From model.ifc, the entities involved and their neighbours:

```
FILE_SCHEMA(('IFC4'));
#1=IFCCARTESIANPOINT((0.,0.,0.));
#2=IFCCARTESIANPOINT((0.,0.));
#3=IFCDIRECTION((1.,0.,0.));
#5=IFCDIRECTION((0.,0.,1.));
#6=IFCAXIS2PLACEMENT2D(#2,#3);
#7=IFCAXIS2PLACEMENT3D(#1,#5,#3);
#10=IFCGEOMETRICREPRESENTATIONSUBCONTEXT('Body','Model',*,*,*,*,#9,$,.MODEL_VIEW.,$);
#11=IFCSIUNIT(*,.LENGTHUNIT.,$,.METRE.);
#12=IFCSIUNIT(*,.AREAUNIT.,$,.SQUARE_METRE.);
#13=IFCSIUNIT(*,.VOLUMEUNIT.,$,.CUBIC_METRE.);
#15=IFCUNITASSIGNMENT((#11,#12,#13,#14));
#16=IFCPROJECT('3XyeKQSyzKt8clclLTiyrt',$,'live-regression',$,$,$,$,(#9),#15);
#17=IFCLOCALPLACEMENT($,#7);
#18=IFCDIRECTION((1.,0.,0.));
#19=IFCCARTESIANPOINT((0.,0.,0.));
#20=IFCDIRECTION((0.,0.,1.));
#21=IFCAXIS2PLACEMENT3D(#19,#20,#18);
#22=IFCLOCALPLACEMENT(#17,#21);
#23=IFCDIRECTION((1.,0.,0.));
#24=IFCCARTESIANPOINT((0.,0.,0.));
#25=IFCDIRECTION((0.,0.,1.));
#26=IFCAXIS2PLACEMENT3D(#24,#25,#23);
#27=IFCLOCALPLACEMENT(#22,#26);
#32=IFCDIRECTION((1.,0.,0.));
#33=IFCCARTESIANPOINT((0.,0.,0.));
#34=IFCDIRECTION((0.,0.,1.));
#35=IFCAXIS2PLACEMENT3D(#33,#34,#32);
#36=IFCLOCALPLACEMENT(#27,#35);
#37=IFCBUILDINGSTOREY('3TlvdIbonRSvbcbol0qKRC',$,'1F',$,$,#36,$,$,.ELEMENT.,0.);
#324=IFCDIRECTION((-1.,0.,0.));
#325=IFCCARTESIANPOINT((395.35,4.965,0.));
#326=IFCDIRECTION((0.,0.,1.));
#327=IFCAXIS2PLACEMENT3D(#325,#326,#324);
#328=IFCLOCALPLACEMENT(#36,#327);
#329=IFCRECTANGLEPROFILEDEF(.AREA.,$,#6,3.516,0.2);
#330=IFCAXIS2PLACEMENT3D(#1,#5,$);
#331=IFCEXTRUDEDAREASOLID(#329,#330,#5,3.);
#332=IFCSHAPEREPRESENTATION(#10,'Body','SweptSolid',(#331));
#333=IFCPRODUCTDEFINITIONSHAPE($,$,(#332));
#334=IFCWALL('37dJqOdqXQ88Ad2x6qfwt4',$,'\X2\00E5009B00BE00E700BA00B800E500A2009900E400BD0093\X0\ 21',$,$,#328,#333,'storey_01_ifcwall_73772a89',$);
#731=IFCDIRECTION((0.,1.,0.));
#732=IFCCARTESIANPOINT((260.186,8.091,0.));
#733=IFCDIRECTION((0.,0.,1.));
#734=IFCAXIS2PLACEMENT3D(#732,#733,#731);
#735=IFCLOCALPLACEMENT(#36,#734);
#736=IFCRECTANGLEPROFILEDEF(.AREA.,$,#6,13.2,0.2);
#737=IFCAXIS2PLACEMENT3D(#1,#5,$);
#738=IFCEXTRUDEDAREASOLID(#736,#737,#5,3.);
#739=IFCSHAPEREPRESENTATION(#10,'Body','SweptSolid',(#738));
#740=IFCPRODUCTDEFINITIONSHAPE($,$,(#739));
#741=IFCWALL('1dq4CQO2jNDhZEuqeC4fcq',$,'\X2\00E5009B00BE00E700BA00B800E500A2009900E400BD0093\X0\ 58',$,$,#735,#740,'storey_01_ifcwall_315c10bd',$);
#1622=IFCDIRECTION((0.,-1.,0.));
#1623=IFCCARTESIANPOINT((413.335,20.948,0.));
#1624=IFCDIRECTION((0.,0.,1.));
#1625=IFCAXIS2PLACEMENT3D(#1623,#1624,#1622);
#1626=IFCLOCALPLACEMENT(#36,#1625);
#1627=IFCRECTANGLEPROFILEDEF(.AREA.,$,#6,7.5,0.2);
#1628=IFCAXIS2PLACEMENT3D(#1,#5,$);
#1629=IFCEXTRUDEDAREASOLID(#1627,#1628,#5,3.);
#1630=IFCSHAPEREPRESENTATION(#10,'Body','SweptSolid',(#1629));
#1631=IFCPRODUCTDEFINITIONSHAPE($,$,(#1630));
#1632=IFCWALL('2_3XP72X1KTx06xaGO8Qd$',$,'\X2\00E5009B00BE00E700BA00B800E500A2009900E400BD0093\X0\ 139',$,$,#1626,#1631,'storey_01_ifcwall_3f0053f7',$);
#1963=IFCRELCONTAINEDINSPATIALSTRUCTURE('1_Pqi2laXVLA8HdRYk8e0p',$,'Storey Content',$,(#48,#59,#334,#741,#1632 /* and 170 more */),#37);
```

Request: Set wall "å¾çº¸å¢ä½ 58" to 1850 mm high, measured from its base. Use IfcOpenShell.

```python
import ifcopenshell
import ifcopenshell.geom
import ifcopenshell.util.representation
import ifcopenshell.util.shape
import ifcopenshell.util.unit

model = ifcopenshell.open("model.ifc")
unit_scale = ifcopenshell.util.unit.calculate_unit_scale(model)
settings = ifcopenshell.geom.settings()


def volume(element):
    """Net volume in cubic metres, openings subtracted."""
    shape = ifcopenshell.geom.create_shape(settings, element)
    return ifcopenshell.util.shape.get_volume(shape.geometry)


wall = model.by_id(741)
before = volume(wall)

body = ifcopenshell.util.representation.get_representation(wall, "Model", "Body")
solid = body.Items[0]
old_height = solid.Depth
solid.Depth = 1.85 / unit_scale
after = volume(wall)

print(f"height {old_height:g} -> {solid.Depth:g}, volume {before:.3f} -> {after:.3f} m3")

model.write("model_v2.ifc")
```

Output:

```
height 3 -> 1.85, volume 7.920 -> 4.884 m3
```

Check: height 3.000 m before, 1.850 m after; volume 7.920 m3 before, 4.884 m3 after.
